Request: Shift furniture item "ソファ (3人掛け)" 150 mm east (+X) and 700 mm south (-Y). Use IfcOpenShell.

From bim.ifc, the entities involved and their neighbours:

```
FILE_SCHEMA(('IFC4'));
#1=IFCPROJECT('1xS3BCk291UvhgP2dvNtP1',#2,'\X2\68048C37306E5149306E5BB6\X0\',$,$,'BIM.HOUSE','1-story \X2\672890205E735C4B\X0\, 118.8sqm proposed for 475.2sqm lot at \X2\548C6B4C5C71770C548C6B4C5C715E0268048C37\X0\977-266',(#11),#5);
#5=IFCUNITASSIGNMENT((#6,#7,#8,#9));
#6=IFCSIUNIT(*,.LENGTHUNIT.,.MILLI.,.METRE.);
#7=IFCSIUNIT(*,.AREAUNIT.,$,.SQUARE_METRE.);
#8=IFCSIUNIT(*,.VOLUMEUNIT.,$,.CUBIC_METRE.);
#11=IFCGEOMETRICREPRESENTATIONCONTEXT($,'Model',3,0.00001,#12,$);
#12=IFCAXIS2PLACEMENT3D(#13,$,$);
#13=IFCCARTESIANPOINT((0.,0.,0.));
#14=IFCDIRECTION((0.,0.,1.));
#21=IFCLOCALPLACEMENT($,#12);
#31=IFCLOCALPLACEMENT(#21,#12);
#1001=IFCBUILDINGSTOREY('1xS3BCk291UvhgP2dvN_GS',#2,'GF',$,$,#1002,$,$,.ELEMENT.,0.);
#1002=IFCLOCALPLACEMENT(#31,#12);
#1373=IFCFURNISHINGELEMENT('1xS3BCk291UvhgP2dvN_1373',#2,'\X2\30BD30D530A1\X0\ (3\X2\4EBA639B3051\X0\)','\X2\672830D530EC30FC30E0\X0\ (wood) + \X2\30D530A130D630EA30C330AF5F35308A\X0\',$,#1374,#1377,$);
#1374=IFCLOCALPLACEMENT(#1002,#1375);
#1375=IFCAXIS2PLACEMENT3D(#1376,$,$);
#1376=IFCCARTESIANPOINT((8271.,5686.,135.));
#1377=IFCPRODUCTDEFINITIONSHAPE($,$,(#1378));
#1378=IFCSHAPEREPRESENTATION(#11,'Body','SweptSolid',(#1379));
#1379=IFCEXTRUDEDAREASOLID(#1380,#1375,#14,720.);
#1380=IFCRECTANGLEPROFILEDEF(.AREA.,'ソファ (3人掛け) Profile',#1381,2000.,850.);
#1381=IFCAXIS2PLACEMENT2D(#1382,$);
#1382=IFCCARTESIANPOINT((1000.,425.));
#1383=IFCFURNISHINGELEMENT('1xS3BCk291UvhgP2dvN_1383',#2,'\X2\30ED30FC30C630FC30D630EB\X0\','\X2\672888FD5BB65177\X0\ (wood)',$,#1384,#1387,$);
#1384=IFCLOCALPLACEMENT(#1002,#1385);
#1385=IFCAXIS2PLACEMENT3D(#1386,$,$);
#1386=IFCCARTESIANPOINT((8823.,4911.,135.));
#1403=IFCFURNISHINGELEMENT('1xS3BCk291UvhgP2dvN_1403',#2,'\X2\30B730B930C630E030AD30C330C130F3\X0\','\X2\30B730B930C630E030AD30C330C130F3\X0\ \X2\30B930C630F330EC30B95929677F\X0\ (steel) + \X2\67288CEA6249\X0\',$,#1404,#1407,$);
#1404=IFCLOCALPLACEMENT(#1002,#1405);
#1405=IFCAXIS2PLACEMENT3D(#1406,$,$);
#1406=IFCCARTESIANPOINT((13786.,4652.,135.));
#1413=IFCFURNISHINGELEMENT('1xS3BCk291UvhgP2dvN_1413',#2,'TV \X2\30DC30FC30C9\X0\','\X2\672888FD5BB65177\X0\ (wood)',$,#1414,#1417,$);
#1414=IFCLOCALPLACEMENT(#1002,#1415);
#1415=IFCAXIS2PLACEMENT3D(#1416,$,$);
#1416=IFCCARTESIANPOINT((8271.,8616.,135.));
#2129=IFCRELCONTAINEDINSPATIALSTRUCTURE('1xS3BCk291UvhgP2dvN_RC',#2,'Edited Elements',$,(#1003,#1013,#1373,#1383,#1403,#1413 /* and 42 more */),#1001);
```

```python
import ifcopenshell
import ifcopenshell.api.geometry
import ifcopenshell.util.placement
import ifcopenshell.util.unit

model = ifcopenshell.open("bim.ifc")
unit_scale = ifcopenshell.util.unit.calculate_unit_scale(model)

item = model.by_id(1373)
matrix = ifcopenshell.util.placement.get_local_placement(item.ObjectPlacement)
matrix[0, 3] += 0.15 / unit_scale
matrix[1, 3] -= 0.7 / unit_scale
ifcopenshell.api.geometry.edit_object_placement(model, product=item, matrix=matrix, is_si=False)

print(ifcopenshell.util.placement.get_local_placement(item.ObjectPlacement).round(3) + 0.0)

model.write("bim_updated.ifc")
```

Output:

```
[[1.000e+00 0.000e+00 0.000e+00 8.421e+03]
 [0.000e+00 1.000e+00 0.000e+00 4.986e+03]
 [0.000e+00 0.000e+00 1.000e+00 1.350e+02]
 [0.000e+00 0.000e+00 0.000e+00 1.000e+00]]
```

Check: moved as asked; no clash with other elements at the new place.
